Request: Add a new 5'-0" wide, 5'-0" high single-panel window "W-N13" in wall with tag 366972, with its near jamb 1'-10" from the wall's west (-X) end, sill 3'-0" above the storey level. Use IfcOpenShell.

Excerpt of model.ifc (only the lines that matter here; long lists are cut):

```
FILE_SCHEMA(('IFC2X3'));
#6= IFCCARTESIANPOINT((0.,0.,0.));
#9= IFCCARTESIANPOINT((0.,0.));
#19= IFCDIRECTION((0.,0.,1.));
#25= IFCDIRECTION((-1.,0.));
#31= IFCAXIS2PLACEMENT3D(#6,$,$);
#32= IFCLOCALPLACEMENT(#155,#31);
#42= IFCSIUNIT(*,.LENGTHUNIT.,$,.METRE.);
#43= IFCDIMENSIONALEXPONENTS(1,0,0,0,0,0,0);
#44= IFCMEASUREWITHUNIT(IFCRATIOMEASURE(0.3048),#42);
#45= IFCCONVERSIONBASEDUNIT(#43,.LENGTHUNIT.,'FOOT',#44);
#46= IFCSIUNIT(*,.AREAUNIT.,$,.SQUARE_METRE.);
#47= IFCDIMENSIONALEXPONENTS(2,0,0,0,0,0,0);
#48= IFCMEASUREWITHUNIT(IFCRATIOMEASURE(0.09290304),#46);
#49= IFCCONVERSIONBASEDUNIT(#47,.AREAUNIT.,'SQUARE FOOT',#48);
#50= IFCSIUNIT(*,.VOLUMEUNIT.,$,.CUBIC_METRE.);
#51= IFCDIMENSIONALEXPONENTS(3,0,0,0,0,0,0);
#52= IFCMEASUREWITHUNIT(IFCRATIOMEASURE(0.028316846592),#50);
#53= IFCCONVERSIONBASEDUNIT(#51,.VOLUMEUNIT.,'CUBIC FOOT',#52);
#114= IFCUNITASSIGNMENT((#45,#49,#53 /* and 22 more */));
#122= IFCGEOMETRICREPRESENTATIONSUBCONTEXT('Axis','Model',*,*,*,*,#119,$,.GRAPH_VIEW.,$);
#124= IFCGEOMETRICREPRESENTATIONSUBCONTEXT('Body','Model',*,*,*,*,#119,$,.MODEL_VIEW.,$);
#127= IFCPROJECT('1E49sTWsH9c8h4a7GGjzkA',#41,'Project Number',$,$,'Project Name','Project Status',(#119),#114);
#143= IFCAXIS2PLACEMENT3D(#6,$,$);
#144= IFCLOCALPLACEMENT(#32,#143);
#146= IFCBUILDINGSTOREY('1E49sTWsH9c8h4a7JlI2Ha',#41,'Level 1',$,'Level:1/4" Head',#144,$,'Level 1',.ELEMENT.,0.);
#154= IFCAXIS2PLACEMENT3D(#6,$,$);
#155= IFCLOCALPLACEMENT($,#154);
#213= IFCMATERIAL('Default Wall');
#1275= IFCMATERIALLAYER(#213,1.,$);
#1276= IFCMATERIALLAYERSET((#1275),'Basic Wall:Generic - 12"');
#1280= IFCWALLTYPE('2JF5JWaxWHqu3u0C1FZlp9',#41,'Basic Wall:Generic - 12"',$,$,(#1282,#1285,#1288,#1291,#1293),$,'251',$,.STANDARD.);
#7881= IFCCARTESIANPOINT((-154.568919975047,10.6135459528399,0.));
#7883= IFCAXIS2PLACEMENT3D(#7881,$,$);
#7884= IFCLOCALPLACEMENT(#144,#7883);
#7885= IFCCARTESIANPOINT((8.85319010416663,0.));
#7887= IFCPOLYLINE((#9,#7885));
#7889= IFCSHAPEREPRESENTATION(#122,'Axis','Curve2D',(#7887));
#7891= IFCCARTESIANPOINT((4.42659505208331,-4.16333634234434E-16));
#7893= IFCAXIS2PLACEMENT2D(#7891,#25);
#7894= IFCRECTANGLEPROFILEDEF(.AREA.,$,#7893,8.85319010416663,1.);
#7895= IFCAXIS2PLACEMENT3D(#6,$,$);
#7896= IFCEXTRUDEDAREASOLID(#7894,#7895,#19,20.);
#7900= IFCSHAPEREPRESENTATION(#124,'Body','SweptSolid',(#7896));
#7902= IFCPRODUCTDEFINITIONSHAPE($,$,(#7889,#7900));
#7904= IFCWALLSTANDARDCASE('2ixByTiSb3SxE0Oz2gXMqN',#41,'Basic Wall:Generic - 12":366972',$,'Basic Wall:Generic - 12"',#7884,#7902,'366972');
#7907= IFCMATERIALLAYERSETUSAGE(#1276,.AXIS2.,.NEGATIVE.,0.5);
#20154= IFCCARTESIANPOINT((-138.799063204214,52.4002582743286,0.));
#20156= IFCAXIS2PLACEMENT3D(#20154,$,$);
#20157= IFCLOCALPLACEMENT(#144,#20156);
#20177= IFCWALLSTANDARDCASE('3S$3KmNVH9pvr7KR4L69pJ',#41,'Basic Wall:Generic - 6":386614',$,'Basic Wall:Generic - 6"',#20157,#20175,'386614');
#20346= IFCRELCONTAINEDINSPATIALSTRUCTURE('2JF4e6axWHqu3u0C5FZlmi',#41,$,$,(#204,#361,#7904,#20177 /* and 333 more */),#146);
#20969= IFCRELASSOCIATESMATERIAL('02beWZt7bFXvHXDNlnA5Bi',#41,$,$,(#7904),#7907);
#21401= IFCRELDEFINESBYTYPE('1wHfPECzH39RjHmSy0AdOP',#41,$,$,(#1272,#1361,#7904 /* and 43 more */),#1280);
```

```python
import numpy as np
import ifcopenshell
import ifcopenshell.api.feature
import ifcopenshell.api.geometry
import ifcopenshell.api.root
import ifcopenshell.api.spatial
import ifcopenshell.api.type
import ifcopenshell.geom
import ifcopenshell.util.element
import ifcopenshell.util.placement
import ifcopenshell.util.representation
import ifcopenshell.util.shape
import ifcopenshell.util.unit

model = ifcopenshell.open("model.ifc")
unit_scale = ifcopenshell.util.unit.calculate_unit_scale(model)
settings = ifcopenshell.geom.settings()


def volume(element):
    """Net volume in cubic metres, openings subtracted."""
    shape = ifcopenshell.geom.create_shape(settings, element)
    return ifcopenshell.util.shape.get_volume(shape.geometry)


wall = model.by_guid("2ixByTiSb3SxE0Oz2gXMqN")
storey = ifcopenshell.util.element.get_container(wall, ifc_class="IfcBuildingStorey")
context = ifcopenshell.util.representation.get_context(model, "Model", "Body", "MODEL_VIEW")
before = volume(wall)

width, height, from_end, sill = 1.524, 1.524, 0.5588, 0.9144  # metres

# The wall runs along its own X axis, and the end named is its -X end.
wall_shape = ifcopenshell.geom.create_shape(settings, wall)
x, y, z = ifcopenshell.util.shape.get_vertices(wall_shape.geometry).T
start = x.min() + from_end
face, thickness = float(y.min()), float(y.max() - y.min())
wall_matrix = ifcopenshell.util.placement.get_local_placement(wall.ObjectPlacement)
level = ifcopenshell.util.placement.get_local_placement(storey.ObjectPlacement)[2, 3]


def in_wall(x, y):
    """Placement at x, y metres in the wall's axes, at sill height."""
    matrix = wall_matrix.copy()
    matrix[:, 3] = wall_matrix @ np.array([x / unit_scale, y / unit_scale, 0.0, 1.0])
    matrix[2, 3] = level + sill / unit_scale
    return matrix


# Opening: a box that overshoots both wall faces by 50 mm.
opening = ifcopenshell.api.root.create_entity(model, ifc_class="IfcOpeningElement")
box = ifcopenshell.api.geometry.add_wall_representation(
    model, context=context, length=width, height=height, thickness=thickness + 0.1
)
ifcopenshell.api.geometry.assign_representation(model, product=opening, representation=box)
ifcopenshell.api.geometry.edit_object_placement(model, product=opening, matrix=in_wall(start, face - 0.05), is_si=False)
ifcopenshell.api.feature.add_feature(model, feature=opening, element=wall)

window = ifcopenshell.api.root.create_entity(model, ifc_class="IfcWindow", name="W-N13")
window.OverallWidth, window.OverallHeight = width / unit_scale, height / unit_scale
body = ifcopenshell.api.geometry.add_window_representation(
    model,
    context=context,
    overall_width=window.OverallWidth,
    overall_height=window.OverallHeight,
    partition_type="SINGLE_PANEL",
)
ifcopenshell.api.geometry.assign_representation(model, product=window, representation=body)
ifcopenshell.api.spatial.assign_container(model, products=[window], relating_structure=storey)
fills = ifcopenshell.api.feature.add_filling(model, opening=opening, element=window)
fills.OwnerHistory = window.OwnerHistory  # required in IFC2X3

# IFC2X3 keeps the operation on the window style.
style = ifcopenshell.api.root.create_entity(model, ifc_class="IfcWindowStyle", name="W-N13")
style.OperationType, style.ConstructionType = "SINGLE_PANEL", "NOTDEFINED"
style.ParameterTakesPrecedence = style.Sizeable = False
ifcopenshell.api.type.assign_type(model, related_objects=[window], relating_type=style)

# Centre the window in the wall's thickness.
ifcopenshell.api.geometry.edit_object_placement(model, product=window, matrix=in_wall(start, face), is_si=False)
window_shape = ifcopenshell.geom.create_shape(settings, window)
depth = ifcopenshell.util.shape.get_vertices(window_shape.geometry)[:, 1]
offset = face + thickness / 2 - (depth.min() + depth.max()) / 2
ifcopenshell.api.geometry.edit_object_placement(model, product=window, matrix=in_wall(start, offset), is_si=False)

after = volume(wall)

print(f"wall volume {before:.3f} -> {after:.3f} m3")

model.write("model_rev.ifc")
```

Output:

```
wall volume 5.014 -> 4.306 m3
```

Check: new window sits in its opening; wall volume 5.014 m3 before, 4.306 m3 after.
